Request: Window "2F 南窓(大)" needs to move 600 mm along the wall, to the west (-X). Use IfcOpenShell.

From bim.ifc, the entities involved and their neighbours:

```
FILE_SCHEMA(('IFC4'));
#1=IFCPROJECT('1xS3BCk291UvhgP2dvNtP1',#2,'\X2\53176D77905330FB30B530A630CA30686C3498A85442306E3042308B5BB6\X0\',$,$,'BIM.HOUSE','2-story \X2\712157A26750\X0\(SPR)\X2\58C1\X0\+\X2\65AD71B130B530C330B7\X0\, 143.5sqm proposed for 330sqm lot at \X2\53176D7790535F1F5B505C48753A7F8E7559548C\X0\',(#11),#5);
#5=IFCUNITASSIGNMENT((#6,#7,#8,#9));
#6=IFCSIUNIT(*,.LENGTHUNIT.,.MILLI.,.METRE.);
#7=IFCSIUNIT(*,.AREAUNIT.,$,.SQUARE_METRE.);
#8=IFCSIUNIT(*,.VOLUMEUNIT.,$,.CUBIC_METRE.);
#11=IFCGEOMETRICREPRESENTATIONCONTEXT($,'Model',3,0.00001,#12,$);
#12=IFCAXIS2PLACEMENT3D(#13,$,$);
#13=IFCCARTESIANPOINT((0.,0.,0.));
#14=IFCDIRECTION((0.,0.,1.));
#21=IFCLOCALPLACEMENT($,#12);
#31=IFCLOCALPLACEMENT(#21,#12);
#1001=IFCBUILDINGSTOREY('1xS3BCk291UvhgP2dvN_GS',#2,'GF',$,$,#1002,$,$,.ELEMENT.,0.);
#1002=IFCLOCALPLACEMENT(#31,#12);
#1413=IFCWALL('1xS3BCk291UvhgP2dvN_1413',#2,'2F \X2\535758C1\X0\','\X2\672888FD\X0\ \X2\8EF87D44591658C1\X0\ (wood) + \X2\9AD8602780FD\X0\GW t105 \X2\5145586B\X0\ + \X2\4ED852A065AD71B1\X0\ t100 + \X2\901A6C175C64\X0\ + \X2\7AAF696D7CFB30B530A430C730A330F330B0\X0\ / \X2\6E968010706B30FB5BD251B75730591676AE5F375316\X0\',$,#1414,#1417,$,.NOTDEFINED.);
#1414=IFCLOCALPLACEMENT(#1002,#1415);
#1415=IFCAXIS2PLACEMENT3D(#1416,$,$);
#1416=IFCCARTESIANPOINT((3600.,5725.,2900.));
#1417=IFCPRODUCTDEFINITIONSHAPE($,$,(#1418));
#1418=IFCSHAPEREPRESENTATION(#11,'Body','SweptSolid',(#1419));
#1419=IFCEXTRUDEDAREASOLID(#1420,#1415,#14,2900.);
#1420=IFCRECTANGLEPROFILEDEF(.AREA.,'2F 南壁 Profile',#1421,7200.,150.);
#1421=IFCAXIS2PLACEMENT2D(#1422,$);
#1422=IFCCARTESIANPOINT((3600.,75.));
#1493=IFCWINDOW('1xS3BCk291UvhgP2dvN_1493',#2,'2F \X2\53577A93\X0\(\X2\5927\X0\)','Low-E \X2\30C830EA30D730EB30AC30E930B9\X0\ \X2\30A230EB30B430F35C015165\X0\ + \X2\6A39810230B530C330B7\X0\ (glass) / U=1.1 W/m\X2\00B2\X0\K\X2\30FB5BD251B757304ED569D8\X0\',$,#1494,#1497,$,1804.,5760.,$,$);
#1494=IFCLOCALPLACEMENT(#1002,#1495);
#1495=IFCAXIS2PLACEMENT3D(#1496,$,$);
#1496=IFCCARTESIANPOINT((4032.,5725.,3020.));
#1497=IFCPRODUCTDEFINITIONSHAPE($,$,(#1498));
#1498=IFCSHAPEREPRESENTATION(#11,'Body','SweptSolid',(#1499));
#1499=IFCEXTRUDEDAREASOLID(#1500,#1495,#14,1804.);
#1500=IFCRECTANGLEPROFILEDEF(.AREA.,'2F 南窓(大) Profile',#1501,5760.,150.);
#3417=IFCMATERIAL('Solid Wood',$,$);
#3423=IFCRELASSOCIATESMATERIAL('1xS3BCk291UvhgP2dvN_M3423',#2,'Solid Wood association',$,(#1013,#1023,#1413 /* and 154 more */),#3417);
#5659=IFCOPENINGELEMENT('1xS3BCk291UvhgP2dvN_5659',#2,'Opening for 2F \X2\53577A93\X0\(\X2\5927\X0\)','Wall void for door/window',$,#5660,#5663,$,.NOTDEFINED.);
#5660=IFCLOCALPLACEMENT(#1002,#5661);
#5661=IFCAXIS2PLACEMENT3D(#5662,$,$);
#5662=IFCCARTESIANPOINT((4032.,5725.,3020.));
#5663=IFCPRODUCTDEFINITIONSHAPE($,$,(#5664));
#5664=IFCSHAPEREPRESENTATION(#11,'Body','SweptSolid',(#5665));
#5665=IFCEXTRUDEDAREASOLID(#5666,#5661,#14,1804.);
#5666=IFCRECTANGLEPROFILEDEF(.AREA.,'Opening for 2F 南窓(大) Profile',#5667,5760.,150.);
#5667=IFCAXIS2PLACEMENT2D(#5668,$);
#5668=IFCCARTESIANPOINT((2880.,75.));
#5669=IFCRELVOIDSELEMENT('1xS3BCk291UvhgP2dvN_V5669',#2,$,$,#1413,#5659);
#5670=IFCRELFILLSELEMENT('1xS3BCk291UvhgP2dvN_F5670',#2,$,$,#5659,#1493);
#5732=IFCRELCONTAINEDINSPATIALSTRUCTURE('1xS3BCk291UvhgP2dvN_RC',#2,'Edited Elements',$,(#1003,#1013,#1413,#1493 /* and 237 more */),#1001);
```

```python
import ifcopenshell
import ifcopenshell.api.geometry
import ifcopenshell.util.placement
import ifcopenshell.util.unit

model = ifcopenshell.open("bim.ifc")
unit_scale = ifcopenshell.util.unit.calculate_unit_scale(model)

window = model.by_guid("1xS3BCk291UvhgP2dvN_1493")
opening = window.FillsVoids[0].RelatingOpeningElement
wall = opening.VoidsElements[0].RelatingBuildingElement

wall_matrix = ifcopenshell.util.placement.get_local_placement(wall.ObjectPlacement)
shift = wall_matrix[:3, 0] * -0.6 / unit_scale
before = ifcopenshell.util.placement.get_local_placement(window.ObjectPlacement)[:3, 3].copy()

# The window is not placed relative to its opening, so move both.
for product in (opening, window):
    matrix = ifcopenshell.util.placement.get_local_placement(product.ObjectPlacement)
    matrix[:3, 3] += shift
    ifcopenshell.api.geometry.edit_object_placement(model, product=product, matrix=matrix, is_si=False)

after = ifcopenshell.util.placement.get_local_placement(window.ObjectPlacement)[:3, 3]
print("window moved by", (after - before).round(3) + 0.0)

model.write("bim_v2.ifc")
```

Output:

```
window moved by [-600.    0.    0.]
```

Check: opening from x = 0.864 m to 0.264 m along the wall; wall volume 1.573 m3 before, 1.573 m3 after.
